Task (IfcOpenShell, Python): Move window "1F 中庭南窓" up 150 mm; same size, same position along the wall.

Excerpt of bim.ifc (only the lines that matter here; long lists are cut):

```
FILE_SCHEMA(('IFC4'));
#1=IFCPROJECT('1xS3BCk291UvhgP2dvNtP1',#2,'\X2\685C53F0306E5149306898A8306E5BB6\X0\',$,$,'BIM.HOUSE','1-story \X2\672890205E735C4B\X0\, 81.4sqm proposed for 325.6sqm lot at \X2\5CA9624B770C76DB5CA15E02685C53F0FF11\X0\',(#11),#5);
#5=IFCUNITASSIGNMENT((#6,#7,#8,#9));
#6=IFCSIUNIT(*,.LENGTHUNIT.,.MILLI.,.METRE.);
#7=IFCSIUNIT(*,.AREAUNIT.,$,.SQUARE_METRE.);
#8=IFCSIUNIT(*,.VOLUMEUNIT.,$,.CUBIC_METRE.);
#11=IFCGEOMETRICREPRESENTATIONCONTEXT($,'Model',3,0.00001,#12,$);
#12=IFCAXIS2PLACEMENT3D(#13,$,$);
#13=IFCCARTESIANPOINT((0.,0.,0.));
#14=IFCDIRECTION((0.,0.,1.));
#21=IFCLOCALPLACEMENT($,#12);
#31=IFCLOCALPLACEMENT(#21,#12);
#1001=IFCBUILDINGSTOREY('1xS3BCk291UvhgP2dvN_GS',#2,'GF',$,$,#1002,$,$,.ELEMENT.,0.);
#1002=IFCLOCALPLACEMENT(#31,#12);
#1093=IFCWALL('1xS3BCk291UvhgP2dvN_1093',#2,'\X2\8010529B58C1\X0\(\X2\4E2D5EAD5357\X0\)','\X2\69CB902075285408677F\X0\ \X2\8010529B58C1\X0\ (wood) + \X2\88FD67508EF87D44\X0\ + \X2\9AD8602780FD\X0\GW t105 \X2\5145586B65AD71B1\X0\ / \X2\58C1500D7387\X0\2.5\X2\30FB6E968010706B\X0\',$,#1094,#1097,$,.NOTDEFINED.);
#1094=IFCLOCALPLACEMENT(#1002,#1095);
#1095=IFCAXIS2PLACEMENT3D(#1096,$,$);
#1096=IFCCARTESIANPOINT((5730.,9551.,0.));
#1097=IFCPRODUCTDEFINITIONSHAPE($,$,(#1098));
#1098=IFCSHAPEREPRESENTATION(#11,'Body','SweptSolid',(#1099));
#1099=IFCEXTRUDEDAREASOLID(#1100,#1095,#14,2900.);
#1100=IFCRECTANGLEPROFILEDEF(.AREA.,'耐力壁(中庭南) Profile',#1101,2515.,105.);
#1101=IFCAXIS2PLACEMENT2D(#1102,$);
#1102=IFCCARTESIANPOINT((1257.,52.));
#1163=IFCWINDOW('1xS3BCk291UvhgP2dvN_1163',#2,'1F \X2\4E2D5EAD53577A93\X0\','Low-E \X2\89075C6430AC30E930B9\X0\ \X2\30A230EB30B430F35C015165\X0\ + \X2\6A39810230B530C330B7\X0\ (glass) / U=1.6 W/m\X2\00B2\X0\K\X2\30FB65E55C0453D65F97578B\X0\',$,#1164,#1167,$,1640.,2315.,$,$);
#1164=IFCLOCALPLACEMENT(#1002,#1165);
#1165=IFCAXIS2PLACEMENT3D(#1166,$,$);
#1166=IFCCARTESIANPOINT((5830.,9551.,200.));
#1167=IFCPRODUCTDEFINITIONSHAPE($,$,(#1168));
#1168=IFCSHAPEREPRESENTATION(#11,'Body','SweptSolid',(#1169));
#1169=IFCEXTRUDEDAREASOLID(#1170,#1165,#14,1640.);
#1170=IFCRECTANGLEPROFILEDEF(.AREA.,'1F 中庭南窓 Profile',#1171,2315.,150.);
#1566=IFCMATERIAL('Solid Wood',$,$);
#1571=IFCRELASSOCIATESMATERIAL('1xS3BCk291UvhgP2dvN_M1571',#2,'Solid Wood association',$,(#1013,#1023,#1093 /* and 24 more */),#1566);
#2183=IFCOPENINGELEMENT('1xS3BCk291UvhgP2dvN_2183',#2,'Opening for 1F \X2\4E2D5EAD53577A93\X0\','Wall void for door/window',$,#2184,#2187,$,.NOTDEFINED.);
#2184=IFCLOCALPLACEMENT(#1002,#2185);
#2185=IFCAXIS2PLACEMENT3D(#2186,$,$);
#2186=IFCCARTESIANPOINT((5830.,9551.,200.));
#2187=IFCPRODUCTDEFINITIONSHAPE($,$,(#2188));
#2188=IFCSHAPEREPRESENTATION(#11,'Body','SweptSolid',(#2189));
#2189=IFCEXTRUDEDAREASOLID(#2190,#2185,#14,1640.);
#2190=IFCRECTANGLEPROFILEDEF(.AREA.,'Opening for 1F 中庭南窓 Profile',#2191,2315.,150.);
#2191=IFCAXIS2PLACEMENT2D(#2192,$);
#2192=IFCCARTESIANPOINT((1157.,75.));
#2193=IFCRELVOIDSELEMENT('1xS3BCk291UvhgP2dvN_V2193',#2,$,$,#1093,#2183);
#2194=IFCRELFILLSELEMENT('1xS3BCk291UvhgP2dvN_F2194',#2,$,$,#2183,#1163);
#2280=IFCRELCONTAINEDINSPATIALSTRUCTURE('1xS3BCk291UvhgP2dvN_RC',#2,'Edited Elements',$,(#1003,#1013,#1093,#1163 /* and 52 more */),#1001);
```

```python
import numpy as np
import ifcopenshell
import ifcopenshell.api.geometry
import ifcopenshell.util.placement
import ifcopenshell.util.unit

model = ifcopenshell.open("bim.ifc")
unit_scale = ifcopenshell.util.unit.calculate_unit_scale(model)

window = model.by_id(1163)
opening = window.FillsVoids[0].RelatingOpeningElement
dz = 0.15 / unit_scale

shift = np.array([0.0, 0.0, dz])
# The window is not placed relative to its opening, so move both.
for product in (opening, window):
    matrix = ifcopenshell.util.placement.get_local_placement(product.ObjectPlacement)
    matrix[:3, 3] += shift
    ifcopenshell.api.geometry.edit_object_placement(model, product=product, matrix=matrix, is_si=False)

print(f"moved by {dz * unit_scale:+.3f} m")

model.write("bim-out.ifc")
```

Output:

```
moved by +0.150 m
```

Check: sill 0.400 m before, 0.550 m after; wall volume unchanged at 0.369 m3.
